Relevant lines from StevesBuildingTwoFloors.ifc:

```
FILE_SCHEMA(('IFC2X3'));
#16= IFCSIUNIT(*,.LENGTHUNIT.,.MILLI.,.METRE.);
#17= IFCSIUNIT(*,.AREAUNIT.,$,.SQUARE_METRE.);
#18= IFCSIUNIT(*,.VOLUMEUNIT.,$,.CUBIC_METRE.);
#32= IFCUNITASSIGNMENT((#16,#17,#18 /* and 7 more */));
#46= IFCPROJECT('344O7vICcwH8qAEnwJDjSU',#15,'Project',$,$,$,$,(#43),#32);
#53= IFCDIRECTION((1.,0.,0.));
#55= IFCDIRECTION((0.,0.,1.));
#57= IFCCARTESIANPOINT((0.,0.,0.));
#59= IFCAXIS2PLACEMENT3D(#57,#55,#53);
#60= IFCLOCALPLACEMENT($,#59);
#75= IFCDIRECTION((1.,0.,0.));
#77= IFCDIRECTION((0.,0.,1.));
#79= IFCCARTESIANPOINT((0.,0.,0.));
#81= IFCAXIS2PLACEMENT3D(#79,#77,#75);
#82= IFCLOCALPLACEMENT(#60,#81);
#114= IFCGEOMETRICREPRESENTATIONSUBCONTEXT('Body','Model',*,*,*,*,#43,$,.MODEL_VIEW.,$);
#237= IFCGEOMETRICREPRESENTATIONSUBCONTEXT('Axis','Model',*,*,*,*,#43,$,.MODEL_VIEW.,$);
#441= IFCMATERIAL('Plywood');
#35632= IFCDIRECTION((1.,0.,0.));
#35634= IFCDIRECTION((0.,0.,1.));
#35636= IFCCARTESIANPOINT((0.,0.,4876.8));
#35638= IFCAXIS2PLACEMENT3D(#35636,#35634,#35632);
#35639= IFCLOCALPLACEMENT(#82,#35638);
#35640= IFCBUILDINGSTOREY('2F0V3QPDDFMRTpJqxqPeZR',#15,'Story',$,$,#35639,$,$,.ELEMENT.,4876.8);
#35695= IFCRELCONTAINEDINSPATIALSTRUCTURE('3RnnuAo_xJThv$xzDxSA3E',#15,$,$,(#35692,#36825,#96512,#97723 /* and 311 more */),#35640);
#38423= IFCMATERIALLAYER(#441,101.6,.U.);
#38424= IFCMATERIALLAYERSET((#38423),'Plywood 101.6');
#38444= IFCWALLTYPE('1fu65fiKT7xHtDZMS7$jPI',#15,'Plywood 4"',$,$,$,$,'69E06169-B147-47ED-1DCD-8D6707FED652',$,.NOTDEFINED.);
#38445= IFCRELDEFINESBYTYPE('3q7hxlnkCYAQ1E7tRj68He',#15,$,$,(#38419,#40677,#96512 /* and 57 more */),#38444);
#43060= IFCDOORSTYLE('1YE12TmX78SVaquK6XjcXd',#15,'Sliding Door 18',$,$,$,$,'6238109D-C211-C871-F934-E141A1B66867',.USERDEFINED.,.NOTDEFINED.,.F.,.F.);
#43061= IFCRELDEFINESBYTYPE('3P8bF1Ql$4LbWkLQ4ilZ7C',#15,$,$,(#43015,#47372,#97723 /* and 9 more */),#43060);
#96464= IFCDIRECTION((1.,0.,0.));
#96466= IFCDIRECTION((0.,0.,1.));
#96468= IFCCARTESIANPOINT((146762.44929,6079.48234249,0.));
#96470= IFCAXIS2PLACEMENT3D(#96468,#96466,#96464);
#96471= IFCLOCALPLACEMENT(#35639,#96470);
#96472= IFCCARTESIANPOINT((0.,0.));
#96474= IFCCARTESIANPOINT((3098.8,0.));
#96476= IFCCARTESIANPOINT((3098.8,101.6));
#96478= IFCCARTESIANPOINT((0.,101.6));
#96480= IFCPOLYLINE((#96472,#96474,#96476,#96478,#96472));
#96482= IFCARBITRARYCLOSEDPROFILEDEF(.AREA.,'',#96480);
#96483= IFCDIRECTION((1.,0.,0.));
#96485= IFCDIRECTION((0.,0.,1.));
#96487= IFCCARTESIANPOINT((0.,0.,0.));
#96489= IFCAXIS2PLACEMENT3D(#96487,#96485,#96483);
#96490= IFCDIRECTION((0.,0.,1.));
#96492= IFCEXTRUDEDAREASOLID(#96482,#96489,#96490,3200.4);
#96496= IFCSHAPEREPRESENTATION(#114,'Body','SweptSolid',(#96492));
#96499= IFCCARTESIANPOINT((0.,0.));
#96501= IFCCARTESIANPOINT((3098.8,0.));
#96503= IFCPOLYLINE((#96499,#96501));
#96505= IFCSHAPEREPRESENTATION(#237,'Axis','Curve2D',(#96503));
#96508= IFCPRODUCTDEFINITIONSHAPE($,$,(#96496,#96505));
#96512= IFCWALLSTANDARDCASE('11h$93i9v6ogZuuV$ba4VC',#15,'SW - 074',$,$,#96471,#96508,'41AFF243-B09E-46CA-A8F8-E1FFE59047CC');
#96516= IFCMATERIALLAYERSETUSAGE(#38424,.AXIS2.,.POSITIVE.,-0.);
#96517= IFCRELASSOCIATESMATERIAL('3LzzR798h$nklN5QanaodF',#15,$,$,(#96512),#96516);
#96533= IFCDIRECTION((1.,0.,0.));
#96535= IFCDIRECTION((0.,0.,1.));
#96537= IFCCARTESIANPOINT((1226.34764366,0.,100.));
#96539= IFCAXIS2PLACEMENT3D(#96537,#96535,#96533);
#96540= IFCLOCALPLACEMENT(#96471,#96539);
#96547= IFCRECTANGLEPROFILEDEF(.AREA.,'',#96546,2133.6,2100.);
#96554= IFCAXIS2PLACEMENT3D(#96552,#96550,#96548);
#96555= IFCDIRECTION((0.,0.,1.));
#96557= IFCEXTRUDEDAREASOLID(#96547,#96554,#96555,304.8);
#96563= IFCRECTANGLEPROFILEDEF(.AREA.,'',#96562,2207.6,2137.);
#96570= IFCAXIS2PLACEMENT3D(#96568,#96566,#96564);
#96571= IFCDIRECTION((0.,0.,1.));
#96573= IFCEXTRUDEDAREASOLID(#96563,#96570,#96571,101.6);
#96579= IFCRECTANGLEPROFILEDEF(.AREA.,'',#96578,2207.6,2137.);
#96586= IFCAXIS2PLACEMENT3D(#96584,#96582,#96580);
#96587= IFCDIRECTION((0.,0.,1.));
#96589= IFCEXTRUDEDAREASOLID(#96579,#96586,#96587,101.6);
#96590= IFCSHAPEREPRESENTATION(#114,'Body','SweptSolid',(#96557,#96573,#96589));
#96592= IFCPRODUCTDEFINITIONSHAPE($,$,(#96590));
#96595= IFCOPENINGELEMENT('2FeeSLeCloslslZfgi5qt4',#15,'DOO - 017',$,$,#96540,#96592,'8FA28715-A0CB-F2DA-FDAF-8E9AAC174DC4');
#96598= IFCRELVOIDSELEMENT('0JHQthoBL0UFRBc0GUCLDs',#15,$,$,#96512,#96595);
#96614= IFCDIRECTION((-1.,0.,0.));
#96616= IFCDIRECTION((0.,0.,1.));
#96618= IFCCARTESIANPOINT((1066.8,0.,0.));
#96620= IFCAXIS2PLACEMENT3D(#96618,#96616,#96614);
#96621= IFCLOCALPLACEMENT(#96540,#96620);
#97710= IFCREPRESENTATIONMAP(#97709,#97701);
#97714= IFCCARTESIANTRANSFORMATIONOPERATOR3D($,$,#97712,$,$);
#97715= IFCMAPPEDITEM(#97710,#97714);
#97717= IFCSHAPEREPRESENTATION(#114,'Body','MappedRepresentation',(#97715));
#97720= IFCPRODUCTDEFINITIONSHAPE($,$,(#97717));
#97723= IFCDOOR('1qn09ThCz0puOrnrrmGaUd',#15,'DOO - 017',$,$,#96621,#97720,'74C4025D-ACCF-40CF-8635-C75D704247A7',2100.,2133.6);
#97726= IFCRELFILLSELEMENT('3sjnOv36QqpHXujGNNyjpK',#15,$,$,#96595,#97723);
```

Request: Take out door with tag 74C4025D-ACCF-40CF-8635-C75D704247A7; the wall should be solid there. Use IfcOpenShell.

```python
import ifcopenshell
import ifcopenshell.api.feature
import ifcopenshell.api.root
import ifcopenshell.geom
import ifcopenshell.util.shape

model = ifcopenshell.open("StevesBuildingTwoFloors.ifc")
settings = ifcopenshell.geom.settings()


def volume(element):
    """Net volume in cubic metres, openings subtracted."""
    shape = ifcopenshell.geom.create_shape(settings, element)
    return ifcopenshell.util.shape.get_volume(shape.geometry)


door = model.by_guid("1qn09ThCz0puOrnrrmGaUd")
opening = door.FillsVoids[0].RelatingOpeningElement
wall = opening.VoidsElements[0].RelatingBuildingElement
before = volume(wall)

ifcopenshell.api.root.remove_product(model, product=door)
ifcopenshell.api.feature.remove_feature(model, feature=opening)

after = volume(wall)

print(f"wall volume {before:.3f} -> {after:.3f} m3")

model.write("StevesBuildingTwoFloors_edited.ifc")
```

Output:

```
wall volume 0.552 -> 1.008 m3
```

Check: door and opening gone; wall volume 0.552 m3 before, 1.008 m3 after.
